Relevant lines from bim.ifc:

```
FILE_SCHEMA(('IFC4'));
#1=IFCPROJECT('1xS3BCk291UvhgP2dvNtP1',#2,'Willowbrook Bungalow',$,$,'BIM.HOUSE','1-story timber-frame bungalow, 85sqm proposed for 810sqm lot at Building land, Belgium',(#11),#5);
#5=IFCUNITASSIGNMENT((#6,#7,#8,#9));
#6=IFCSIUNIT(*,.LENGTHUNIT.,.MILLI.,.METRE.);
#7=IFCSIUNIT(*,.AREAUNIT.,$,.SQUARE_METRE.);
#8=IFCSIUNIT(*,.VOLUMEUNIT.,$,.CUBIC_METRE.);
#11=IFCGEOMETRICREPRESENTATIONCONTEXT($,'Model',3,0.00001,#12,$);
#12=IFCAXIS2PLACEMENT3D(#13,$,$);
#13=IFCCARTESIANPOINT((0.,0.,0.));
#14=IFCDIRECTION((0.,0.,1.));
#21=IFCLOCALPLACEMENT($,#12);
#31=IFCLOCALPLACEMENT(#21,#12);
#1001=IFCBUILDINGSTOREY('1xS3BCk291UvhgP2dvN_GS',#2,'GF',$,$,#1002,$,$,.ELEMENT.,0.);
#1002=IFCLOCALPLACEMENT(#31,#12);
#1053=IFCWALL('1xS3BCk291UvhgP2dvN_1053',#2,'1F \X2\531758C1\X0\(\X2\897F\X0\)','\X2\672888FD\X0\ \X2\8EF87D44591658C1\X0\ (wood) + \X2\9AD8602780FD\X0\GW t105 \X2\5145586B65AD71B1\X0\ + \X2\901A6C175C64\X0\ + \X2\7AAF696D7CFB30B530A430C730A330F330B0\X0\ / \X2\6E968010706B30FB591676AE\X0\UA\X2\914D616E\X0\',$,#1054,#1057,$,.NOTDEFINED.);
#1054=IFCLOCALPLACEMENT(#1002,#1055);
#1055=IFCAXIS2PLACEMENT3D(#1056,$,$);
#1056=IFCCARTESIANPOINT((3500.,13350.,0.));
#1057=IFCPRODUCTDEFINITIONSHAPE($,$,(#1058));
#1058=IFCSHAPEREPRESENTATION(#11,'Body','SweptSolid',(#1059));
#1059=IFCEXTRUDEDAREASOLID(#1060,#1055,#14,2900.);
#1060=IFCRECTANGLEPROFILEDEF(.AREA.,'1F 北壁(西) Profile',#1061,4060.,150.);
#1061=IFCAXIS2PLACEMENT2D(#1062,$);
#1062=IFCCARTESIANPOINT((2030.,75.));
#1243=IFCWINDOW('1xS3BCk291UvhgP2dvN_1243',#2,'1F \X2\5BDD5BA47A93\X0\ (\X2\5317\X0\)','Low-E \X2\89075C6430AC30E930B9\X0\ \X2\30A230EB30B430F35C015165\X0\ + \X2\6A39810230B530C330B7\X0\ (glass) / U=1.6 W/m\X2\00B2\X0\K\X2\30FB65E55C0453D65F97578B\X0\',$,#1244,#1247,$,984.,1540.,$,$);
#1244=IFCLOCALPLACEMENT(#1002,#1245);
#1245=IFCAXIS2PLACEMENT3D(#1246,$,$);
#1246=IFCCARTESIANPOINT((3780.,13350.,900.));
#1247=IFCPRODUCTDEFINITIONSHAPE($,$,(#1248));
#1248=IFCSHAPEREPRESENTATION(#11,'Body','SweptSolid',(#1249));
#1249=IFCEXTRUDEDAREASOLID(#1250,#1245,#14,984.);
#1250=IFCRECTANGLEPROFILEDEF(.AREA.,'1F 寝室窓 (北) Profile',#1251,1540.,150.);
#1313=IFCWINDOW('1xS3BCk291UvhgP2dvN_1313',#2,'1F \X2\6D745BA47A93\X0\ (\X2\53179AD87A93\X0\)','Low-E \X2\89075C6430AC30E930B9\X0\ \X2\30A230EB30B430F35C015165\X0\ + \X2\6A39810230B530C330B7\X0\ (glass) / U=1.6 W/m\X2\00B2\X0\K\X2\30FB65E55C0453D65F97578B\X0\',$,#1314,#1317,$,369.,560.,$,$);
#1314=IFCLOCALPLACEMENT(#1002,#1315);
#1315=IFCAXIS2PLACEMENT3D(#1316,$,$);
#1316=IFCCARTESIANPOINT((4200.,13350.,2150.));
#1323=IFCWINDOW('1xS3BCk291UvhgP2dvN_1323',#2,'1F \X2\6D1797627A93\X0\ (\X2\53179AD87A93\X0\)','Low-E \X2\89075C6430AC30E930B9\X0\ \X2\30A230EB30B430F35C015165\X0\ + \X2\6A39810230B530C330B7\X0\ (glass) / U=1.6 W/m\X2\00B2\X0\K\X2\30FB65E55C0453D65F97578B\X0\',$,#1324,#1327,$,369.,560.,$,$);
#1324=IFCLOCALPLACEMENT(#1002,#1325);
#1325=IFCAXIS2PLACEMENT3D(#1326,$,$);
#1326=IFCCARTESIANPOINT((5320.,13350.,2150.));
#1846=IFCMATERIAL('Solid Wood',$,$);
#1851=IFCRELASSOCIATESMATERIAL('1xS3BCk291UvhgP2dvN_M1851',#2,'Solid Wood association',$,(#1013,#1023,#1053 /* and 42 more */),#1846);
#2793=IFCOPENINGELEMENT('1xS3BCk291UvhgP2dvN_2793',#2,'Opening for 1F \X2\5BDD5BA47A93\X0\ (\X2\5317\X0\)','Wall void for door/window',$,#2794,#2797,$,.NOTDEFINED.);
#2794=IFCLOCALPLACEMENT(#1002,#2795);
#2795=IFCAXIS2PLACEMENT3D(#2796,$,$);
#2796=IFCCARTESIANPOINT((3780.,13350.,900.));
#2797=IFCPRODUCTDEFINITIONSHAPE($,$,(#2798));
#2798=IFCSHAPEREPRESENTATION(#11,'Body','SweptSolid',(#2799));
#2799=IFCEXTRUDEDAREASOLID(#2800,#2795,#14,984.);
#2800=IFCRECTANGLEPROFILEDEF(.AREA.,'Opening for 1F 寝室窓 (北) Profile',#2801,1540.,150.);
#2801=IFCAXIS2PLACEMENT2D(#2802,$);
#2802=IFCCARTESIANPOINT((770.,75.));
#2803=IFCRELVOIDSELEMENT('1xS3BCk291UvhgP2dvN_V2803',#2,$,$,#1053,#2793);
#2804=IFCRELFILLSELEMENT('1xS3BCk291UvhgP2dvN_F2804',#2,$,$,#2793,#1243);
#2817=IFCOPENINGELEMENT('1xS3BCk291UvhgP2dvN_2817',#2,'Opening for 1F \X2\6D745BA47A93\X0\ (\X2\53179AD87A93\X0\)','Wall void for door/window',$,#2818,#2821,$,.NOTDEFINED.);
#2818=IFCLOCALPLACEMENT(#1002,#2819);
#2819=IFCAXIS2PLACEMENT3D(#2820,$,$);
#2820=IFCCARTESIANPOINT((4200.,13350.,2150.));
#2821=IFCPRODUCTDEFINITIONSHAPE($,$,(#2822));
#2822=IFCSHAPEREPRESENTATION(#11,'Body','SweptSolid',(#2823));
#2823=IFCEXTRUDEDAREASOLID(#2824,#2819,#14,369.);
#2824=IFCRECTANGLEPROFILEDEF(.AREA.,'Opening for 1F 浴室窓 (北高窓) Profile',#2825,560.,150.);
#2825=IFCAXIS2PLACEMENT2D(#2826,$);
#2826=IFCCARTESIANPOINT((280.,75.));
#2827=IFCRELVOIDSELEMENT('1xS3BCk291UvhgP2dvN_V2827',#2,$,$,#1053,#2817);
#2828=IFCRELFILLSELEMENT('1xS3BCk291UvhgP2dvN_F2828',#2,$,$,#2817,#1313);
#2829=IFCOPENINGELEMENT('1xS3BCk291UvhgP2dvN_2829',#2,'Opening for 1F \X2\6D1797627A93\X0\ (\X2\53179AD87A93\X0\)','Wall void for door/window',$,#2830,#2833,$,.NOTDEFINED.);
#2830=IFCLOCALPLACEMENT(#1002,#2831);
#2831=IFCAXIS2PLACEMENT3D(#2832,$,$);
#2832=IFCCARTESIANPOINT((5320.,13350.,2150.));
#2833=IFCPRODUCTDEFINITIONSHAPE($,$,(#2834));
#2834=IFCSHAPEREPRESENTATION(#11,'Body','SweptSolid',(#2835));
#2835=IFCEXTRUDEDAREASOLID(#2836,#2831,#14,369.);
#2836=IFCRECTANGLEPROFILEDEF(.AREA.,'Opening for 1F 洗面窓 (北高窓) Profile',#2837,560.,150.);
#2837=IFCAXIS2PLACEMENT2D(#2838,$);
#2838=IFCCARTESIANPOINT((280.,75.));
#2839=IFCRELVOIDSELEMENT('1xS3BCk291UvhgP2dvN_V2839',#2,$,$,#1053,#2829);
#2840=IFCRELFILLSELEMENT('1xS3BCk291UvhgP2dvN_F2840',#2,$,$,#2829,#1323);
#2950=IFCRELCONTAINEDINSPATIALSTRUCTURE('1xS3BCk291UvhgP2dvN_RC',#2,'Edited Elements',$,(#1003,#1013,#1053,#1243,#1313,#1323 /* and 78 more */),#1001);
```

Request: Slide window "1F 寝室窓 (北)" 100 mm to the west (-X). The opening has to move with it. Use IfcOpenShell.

```python
import ifcopenshell
import ifcopenshell.api.geometry
import ifcopenshell.util.placement
import ifcopenshell.util.unit

model = ifcopenshell.open("bim.ifc")
unit_scale = ifcopenshell.util.unit.calculate_unit_scale(model)

window = model.by_guid("1xS3BCk291UvhgP2dvN_1243")
opening = window.FillsVoids[0].RelatingOpeningElement
wall = opening.VoidsElements[0].RelatingBuildingElement

wall_matrix = ifcopenshell.util.placement.get_local_placement(wall.ObjectPlacement)
shift = wall_matrix[:3, 0] * -0.1 / unit_scale
before = ifcopenshell.util.placement.get_local_placement(window.ObjectPlacement)[:3, 3].copy()

# The window is not placed relative to its opening, so move both.
for product in (opening, window):
    matrix = ifcopenshell.util.placement.get_local_placement(product.ObjectPlacement)
    matrix[:3, 3] += shift
    ifcopenshell.api.geometry.edit_object_placement(model, product=product, matrix=matrix, is_si=False)

after = ifcopenshell.util.placement.get_local_placement(window.ObjectPlacement)[:3, 3]
print("window moved by", (after - before).round(3) + 0.0)

model.write("bim_edited.ifc")
```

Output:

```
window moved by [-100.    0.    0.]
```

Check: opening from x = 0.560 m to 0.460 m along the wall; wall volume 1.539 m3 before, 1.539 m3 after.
